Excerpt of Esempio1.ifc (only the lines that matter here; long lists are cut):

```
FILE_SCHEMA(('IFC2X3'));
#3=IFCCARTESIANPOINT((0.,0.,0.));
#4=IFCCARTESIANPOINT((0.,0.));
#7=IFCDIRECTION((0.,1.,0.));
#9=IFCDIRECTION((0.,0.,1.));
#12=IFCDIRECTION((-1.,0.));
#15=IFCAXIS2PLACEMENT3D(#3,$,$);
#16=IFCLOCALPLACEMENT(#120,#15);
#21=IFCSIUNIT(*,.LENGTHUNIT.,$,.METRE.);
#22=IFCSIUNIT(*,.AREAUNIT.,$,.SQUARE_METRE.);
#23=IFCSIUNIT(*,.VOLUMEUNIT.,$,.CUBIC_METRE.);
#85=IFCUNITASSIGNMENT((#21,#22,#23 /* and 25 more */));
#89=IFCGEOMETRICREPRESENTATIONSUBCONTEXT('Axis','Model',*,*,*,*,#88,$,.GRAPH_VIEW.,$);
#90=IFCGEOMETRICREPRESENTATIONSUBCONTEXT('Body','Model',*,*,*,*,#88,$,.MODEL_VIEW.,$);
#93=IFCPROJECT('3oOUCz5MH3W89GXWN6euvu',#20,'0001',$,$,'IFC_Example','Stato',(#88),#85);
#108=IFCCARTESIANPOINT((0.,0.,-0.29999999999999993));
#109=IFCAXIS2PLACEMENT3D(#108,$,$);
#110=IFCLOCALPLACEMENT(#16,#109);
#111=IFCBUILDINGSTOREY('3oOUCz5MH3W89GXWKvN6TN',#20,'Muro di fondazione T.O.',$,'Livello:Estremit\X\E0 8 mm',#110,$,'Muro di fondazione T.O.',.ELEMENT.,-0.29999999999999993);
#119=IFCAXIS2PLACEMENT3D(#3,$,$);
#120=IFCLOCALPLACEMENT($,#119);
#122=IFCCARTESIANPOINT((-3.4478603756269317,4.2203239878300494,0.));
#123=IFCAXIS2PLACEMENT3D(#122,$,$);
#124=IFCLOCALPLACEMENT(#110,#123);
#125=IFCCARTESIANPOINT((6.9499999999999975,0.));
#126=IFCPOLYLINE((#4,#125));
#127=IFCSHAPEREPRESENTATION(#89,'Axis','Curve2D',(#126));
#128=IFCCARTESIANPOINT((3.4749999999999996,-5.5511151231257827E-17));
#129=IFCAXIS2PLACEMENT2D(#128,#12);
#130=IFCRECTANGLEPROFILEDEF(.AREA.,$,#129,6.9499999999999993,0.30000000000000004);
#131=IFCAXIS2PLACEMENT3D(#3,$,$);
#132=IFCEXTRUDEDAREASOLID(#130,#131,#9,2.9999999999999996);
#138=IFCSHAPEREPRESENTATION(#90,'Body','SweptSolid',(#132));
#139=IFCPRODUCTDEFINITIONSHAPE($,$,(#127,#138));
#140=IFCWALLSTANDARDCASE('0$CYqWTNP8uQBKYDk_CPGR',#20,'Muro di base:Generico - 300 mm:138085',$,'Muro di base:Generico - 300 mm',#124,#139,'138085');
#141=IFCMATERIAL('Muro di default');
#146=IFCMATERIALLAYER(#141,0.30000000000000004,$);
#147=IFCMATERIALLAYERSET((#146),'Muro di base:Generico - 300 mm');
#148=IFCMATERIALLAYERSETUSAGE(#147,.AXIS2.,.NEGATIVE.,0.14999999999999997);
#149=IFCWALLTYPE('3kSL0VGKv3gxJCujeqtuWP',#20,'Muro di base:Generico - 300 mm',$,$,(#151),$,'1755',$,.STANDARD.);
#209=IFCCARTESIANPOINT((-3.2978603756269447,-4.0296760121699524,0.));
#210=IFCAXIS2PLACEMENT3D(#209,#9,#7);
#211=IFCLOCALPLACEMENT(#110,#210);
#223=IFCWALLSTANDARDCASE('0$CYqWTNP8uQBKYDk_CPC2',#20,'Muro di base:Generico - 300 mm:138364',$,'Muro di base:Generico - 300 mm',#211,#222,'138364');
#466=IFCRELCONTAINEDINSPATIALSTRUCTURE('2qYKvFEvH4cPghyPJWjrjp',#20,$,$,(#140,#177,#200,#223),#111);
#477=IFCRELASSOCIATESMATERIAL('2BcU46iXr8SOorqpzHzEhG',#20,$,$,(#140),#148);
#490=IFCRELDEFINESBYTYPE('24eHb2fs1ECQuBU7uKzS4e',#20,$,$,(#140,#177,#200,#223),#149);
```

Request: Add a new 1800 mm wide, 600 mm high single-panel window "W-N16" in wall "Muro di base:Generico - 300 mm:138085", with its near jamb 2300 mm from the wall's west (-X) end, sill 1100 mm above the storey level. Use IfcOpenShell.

```python
import numpy as np
import ifcopenshell
import ifcopenshell.api.feature
import ifcopenshell.api.geometry
import ifcopenshell.api.root
import ifcopenshell.api.spatial
import ifcopenshell.api.type
import ifcopenshell.geom
import ifcopenshell.util.element
import ifcopenshell.util.placement
import ifcopenshell.util.representation
import ifcopenshell.util.shape
import ifcopenshell.util.unit

model = ifcopenshell.open("Esempio1.ifc")
unit_scale = ifcopenshell.util.unit.calculate_unit_scale(model)
settings = ifcopenshell.geom.settings()


def volume(element):
    """Net volume in cubic metres, openings subtracted."""
    shape = ifcopenshell.geom.create_shape(settings, element)
    return ifcopenshell.util.shape.get_volume(shape.geometry)


wall = model.by_guid("0$CYqWTNP8uQBKYDk_CPGR")
storey = ifcopenshell.util.element.get_container(wall, ifc_class="IfcBuildingStorey")
context = ifcopenshell.util.representation.get_context(model, "Model", "Body", "MODEL_VIEW")
before = volume(wall)

width, height, from_end, sill = 1.8, 0.6, 2.3, 1.1  # metres

# The wall runs along its own X axis, and the end named is its -X end.
wall_shape = ifcopenshell.geom.create_shape(settings, wall)
x, y, z = ifcopenshell.util.shape.get_vertices(wall_shape.geometry).T
start = x.min() + from_end
face, thickness = float(y.min()), float(y.max() - y.min())
wall_matrix = ifcopenshell.util.placement.get_local_placement(wall.ObjectPlacement)
level = ifcopenshell.util.placement.get_local_placement(storey.ObjectPlacement)[2, 3]


def in_wall(x, y):
    """Placement at x, y metres in the wall's axes, at sill height."""
    matrix = wall_matrix.copy()
    matrix[:, 3] = wall_matrix @ np.array([x / unit_scale, y / unit_scale, 0.0, 1.0])
    matrix[2, 3] = level + sill / unit_scale
    return matrix


# Opening: a box that overshoots both wall faces by 50 mm.
opening = ifcopenshell.api.root.create_entity(model, ifc_class="IfcOpeningElement")
box = ifcopenshell.api.geometry.add_wall_representation(
    model, context=context, length=width, height=height, thickness=thickness + 0.1
)
ifcopenshell.api.geometry.assign_representation(model, product=opening, representation=box)
ifcopenshell.api.geometry.edit_object_placement(model, product=opening, matrix=in_wall(start, face - 0.05), is_si=False)
ifcopenshell.api.feature.add_feature(model, feature=opening, element=wall)

window = ifcopenshell.api.root.create_entity(model, ifc_class="IfcWindow", name="W-N16")
window.OverallWidth, window.OverallHeight = width / unit_scale, height / unit_scale
body = ifcopenshell.api.geometry.add_window_representation(
    model,
    context=context,
    overall_width=window.OverallWidth,
    overall_height=window.OverallHeight,
    partition_type="SINGLE_PANEL",
)
ifcopenshell.api.geometry.assign_representation(model, product=window, representation=body)
ifcopenshell.api.spatial.assign_container(model, products=[window], relating_structure=storey)
fills = ifcopenshell.api.feature.add_filling(model, opening=opening, element=window)
fills.OwnerHistory = window.OwnerHistory  # required in IFC2X3

# IFC2X3 keeps the operation on the window style.
style = ifcopenshell.api.root.create_entity(model, ifc_class="IfcWindowStyle", name="W-N16")
style.OperationType, style.ConstructionType = "SINGLE_PANEL", "NOTDEFINED"
style.ParameterTakesPrecedence = style.Sizeable = False
ifcopenshell.api.type.assign_type(model, related_objects=[window], relating_type=style)

# Centre the window in the wall's thickness.
ifcopenshell.api.geometry.edit_object_placement(model, product=window, matrix=in_wall(start, face), is_si=False)
window_shape = ifcopenshell.geom.create_shape(settings, window)
depth = ifcopenshell.util.shape.get_vertices(window_shape.geometry)[:, 1]
offset = face + thickness / 2 - (depth.min() + depth.max()) / 2
ifcopenshell.api.geometry.edit_object_placement(model, product=window, matrix=in_wall(start, offset), is_si=False)

after = volume(wall)

print(f"wall volume {before:.3f} -> {after:.3f} m3")

model.write("Esempio1_edited.ifc")
```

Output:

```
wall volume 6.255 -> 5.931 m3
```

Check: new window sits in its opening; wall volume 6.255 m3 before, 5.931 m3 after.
